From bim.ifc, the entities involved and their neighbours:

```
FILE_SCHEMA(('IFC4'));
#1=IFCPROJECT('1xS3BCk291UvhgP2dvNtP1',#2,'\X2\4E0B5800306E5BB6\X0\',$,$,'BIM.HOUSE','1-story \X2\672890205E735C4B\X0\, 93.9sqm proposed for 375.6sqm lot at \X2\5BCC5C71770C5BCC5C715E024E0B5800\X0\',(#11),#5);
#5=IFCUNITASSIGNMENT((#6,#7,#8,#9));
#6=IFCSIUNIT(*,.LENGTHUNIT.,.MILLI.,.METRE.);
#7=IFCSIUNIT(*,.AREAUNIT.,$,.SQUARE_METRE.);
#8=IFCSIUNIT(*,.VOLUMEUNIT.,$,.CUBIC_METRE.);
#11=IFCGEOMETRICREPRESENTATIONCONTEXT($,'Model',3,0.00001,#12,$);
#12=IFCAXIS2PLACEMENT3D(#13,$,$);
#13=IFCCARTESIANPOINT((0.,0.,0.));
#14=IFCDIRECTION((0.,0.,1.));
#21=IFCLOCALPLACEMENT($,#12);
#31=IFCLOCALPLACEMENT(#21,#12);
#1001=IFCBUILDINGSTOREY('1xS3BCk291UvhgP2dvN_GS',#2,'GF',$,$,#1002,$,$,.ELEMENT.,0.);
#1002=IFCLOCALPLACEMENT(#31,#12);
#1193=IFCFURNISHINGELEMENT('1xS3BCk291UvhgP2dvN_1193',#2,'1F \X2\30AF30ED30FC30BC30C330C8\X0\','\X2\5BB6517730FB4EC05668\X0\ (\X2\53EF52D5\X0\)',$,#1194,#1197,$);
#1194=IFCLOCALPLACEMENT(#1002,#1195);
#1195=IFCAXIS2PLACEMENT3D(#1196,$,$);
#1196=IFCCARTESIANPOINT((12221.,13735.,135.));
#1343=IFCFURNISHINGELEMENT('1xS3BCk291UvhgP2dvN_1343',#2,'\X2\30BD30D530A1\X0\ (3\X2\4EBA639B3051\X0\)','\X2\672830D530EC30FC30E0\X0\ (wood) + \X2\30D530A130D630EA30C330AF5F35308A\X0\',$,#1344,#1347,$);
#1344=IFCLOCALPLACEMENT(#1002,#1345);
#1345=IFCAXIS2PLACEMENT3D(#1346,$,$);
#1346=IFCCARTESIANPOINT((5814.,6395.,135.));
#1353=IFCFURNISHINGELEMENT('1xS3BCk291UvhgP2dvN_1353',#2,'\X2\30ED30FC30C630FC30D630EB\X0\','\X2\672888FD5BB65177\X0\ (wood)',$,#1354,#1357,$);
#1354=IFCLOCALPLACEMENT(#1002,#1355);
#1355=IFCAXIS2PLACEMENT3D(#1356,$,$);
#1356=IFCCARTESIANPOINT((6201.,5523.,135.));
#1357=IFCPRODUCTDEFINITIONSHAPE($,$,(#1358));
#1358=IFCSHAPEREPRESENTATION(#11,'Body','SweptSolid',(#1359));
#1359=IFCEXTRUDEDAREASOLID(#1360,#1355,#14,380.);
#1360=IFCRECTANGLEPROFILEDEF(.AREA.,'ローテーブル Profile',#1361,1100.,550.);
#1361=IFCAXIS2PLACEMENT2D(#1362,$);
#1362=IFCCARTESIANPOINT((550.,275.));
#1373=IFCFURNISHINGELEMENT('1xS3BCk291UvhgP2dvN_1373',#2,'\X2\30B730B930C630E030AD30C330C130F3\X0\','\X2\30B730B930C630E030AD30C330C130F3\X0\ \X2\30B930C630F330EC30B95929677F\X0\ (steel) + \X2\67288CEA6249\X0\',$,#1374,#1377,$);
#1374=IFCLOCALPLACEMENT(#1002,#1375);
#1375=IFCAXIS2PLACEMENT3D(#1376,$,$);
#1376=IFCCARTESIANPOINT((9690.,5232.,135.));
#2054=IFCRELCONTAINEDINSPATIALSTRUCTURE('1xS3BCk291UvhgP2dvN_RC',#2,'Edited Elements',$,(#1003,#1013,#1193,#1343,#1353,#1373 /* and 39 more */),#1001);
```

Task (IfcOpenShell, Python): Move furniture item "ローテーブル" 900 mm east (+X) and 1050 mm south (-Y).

```python
import ifcopenshell
import ifcopenshell.api.geometry
import ifcopenshell.util.placement
import ifcopenshell.util.unit

model = ifcopenshell.open("bim.ifc")
unit_scale = ifcopenshell.util.unit.calculate_unit_scale(model)

item = model.by_guid("1xS3BCk291UvhgP2dvN_1353")
matrix = ifcopenshell.util.placement.get_local_placement(item.ObjectPlacement)
matrix[0, 3] += 0.9 / unit_scale
matrix[1, 3] -= 1.05 / unit_scale
ifcopenshell.api.geometry.edit_object_placement(model, product=item, matrix=matrix, is_si=False)

print(ifcopenshell.util.placement.get_local_placement(item.ObjectPlacement).round(3) + 0.0)

model.write("bim_rev.ifc")
```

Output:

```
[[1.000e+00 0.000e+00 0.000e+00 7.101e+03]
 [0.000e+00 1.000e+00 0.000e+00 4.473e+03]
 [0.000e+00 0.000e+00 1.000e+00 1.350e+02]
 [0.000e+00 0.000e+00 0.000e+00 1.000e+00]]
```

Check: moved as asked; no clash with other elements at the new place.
